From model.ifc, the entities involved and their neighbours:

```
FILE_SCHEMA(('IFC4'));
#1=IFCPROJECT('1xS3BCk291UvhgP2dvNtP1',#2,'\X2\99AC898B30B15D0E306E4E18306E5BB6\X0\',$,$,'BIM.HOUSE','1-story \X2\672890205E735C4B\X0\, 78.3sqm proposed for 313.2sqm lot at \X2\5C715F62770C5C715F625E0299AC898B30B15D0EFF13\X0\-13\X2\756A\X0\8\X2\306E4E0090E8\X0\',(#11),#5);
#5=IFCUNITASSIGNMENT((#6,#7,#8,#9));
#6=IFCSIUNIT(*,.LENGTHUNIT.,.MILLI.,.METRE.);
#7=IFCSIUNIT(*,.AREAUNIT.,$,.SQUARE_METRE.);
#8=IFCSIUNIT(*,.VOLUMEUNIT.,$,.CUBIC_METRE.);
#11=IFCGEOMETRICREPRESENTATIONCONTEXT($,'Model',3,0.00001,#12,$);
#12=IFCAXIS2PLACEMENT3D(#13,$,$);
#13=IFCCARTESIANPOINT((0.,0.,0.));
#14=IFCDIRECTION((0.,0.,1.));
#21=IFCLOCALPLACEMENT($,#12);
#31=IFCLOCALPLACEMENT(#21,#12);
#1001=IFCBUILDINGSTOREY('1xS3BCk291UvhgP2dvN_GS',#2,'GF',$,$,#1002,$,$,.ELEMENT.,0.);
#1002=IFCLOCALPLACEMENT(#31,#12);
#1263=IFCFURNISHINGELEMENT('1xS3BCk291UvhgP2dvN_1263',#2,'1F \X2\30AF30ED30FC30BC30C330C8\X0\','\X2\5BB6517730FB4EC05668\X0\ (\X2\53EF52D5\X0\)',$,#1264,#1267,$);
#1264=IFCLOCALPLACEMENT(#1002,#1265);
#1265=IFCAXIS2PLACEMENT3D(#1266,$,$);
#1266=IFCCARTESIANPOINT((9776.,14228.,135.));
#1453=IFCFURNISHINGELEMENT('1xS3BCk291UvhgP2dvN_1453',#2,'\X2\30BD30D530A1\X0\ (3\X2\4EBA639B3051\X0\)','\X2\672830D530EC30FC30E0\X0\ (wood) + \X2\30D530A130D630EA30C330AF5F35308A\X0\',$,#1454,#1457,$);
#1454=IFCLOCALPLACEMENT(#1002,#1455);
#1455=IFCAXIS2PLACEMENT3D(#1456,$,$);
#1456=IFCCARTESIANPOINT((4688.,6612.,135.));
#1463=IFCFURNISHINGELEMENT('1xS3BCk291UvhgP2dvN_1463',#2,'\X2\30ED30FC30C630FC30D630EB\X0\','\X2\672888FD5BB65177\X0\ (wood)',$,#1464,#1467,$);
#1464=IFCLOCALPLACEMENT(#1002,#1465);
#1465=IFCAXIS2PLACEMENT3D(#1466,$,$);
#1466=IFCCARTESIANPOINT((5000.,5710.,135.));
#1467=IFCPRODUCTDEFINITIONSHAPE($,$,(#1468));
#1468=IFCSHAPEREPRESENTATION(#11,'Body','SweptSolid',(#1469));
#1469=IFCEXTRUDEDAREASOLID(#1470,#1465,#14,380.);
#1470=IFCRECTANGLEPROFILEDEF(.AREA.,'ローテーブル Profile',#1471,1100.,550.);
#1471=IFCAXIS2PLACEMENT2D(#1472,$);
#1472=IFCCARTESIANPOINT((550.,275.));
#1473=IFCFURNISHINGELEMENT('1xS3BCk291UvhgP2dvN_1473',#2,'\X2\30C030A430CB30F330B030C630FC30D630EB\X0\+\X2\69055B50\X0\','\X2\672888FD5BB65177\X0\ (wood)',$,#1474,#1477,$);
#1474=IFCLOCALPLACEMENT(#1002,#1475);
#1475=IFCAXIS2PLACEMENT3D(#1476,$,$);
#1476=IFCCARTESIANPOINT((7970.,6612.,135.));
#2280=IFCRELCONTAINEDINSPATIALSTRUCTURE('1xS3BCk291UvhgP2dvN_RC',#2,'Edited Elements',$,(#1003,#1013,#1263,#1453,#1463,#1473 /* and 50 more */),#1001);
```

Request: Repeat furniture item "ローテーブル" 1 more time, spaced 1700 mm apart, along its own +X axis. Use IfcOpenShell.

```python
import ifcopenshell
import ifcopenshell.api.geometry
import ifcopenshell.api.root
import ifcopenshell.util.element
import ifcopenshell.util.placement

model = ifcopenshell.open("model.ifc")


def reuse_history(source, copy):
    """copy_class also copies each property set's owner history, people and application; keep the originals."""
    for rel in copy.IsDefinedBy:
        if rel.is_a("IfcRelDefinesByProperties") and (history := rel.RelatingPropertyDefinition.OwnerHistory):
            rel.RelatingPropertyDefinition.OwnerHistory = source.OwnerHistory
            ifcopenshell.util.element.remove_deep2(model, history)


source = model.by_guid("1xS3BCk291UvhgP2dvN_1463")
base = ifcopenshell.util.placement.get_local_placement(source.ObjectPlacement)
step = base[:3, 0] * 1700.0

for i in range(1, 2):
    copy = ifcopenshell.api.root.copy_class(model, product=source)
    copy.Representation = ifcopenshell.util.element.copy_deep(
        model, source.Representation, exclude=["IfcGeometricRepresentationContext", "IfcRepresentationMap"]
    )
    reuse_history(source, copy)
    matrix = base.copy()
    matrix[:3, 3] += i * step
    print("added at", matrix[:3, 3].round(3) + 0.0)
    ifcopenshell.api.geometry.edit_object_placement(model, product=copy, matrix=matrix, is_si=False)

model.write("model_edited.ifc")
```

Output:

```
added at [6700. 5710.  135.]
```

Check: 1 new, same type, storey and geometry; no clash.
